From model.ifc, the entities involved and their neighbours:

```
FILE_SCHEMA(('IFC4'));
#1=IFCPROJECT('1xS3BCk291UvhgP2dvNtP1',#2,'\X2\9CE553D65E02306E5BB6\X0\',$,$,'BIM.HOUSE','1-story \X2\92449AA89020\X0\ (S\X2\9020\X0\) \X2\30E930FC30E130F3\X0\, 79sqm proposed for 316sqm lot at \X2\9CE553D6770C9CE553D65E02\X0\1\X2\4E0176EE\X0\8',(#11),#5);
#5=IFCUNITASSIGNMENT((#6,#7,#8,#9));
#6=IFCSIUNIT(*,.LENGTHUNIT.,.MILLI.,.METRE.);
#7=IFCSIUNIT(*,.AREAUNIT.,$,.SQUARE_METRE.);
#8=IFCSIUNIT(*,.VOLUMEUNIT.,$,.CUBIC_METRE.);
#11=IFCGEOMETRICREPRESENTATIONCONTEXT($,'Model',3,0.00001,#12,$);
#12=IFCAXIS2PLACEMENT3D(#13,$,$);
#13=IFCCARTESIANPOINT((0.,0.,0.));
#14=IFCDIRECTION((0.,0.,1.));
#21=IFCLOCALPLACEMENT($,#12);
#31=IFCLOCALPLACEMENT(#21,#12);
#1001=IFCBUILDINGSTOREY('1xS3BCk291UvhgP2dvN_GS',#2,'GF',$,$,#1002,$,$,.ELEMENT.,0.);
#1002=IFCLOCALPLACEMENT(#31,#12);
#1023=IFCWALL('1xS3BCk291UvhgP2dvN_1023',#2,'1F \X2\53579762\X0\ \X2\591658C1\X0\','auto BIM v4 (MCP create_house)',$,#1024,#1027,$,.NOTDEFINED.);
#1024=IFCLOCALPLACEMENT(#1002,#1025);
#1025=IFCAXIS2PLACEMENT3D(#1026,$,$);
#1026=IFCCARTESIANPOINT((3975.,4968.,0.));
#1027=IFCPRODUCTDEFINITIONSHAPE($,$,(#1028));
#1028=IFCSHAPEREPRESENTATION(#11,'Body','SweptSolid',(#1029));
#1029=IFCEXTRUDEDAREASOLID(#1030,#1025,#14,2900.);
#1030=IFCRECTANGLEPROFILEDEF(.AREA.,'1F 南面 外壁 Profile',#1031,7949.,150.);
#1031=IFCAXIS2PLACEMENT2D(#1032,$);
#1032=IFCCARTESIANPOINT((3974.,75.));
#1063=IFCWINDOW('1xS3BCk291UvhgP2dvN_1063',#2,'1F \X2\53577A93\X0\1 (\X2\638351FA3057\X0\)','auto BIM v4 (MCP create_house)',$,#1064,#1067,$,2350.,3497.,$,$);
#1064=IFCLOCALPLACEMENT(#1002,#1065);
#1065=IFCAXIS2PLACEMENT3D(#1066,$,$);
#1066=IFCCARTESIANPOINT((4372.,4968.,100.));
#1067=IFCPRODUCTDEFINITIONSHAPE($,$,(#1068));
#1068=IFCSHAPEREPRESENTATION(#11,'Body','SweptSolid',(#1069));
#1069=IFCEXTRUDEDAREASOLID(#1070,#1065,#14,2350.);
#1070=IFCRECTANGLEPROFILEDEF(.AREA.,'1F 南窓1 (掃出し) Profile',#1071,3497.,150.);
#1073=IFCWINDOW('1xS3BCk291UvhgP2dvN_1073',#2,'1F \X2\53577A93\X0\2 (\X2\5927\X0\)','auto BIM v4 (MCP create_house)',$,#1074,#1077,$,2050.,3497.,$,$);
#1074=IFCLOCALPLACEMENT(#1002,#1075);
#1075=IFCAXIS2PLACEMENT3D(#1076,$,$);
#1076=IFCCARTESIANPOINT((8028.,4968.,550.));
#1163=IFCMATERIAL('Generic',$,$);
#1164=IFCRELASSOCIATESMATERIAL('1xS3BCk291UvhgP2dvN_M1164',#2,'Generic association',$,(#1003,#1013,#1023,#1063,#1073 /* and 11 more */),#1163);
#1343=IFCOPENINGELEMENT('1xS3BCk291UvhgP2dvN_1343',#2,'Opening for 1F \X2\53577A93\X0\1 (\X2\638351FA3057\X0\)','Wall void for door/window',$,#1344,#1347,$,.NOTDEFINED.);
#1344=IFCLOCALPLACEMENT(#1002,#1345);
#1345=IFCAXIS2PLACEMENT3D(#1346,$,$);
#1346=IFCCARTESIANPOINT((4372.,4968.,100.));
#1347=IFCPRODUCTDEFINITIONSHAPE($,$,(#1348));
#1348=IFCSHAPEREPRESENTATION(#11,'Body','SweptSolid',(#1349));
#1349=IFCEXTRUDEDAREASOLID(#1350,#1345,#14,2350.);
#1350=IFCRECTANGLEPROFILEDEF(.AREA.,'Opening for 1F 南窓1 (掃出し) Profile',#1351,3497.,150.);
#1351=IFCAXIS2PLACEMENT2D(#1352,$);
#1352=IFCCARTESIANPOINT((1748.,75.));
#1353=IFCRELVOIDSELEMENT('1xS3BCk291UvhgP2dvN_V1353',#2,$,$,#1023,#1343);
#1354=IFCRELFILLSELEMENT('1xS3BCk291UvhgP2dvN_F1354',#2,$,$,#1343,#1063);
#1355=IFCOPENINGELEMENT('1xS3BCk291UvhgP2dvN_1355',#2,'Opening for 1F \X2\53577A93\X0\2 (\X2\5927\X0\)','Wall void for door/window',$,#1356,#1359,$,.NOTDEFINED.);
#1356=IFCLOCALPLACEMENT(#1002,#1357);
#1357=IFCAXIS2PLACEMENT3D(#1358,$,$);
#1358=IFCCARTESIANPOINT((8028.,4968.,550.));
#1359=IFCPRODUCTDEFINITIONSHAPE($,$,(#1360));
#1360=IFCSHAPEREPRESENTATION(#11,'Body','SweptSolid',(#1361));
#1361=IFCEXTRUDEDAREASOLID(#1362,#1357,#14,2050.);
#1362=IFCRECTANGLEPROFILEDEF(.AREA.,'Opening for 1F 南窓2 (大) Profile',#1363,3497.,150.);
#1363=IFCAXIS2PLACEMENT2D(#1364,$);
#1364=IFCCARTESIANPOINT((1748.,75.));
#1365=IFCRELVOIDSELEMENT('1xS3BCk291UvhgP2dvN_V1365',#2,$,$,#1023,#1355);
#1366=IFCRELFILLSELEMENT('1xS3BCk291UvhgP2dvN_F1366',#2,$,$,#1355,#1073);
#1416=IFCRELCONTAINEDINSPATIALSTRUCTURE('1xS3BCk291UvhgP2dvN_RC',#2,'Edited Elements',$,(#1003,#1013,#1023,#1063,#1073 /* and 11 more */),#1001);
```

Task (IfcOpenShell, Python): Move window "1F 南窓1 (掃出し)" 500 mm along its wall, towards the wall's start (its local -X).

```python
import ifcopenshell
import ifcopenshell.api.geometry
import ifcopenshell.util.placement
import ifcopenshell.util.unit

model = ifcopenshell.open("model.ifc")
unit_scale = ifcopenshell.util.unit.calculate_unit_scale(model)

window = model.by_id(1063)
opening = window.FillsVoids[0].RelatingOpeningElement
wall = opening.VoidsElements[0].RelatingBuildingElement

wall_matrix = ifcopenshell.util.placement.get_local_placement(wall.ObjectPlacement)
shift = wall_matrix[:3, 0] * -0.5 / unit_scale
before = ifcopenshell.util.placement.get_local_placement(window.ObjectPlacement)[:3, 3].copy()

# The window is not placed relative to its opening, so move both.
for product in (opening, window):
    matrix = ifcopenshell.util.placement.get_local_placement(product.ObjectPlacement)
    matrix[:3, 3] += shift
    ifcopenshell.api.geometry.edit_object_placement(model, product=product, matrix=matrix, is_si=False)

after = ifcopenshell.util.placement.get_local_placement(window.ObjectPlacement)[:3, 3]
print("window moved by", (after - before).round(3) + 0.0)

model.write("model_rev.ifc")
```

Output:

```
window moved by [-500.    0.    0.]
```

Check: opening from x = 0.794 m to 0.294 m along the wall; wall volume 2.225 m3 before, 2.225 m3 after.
